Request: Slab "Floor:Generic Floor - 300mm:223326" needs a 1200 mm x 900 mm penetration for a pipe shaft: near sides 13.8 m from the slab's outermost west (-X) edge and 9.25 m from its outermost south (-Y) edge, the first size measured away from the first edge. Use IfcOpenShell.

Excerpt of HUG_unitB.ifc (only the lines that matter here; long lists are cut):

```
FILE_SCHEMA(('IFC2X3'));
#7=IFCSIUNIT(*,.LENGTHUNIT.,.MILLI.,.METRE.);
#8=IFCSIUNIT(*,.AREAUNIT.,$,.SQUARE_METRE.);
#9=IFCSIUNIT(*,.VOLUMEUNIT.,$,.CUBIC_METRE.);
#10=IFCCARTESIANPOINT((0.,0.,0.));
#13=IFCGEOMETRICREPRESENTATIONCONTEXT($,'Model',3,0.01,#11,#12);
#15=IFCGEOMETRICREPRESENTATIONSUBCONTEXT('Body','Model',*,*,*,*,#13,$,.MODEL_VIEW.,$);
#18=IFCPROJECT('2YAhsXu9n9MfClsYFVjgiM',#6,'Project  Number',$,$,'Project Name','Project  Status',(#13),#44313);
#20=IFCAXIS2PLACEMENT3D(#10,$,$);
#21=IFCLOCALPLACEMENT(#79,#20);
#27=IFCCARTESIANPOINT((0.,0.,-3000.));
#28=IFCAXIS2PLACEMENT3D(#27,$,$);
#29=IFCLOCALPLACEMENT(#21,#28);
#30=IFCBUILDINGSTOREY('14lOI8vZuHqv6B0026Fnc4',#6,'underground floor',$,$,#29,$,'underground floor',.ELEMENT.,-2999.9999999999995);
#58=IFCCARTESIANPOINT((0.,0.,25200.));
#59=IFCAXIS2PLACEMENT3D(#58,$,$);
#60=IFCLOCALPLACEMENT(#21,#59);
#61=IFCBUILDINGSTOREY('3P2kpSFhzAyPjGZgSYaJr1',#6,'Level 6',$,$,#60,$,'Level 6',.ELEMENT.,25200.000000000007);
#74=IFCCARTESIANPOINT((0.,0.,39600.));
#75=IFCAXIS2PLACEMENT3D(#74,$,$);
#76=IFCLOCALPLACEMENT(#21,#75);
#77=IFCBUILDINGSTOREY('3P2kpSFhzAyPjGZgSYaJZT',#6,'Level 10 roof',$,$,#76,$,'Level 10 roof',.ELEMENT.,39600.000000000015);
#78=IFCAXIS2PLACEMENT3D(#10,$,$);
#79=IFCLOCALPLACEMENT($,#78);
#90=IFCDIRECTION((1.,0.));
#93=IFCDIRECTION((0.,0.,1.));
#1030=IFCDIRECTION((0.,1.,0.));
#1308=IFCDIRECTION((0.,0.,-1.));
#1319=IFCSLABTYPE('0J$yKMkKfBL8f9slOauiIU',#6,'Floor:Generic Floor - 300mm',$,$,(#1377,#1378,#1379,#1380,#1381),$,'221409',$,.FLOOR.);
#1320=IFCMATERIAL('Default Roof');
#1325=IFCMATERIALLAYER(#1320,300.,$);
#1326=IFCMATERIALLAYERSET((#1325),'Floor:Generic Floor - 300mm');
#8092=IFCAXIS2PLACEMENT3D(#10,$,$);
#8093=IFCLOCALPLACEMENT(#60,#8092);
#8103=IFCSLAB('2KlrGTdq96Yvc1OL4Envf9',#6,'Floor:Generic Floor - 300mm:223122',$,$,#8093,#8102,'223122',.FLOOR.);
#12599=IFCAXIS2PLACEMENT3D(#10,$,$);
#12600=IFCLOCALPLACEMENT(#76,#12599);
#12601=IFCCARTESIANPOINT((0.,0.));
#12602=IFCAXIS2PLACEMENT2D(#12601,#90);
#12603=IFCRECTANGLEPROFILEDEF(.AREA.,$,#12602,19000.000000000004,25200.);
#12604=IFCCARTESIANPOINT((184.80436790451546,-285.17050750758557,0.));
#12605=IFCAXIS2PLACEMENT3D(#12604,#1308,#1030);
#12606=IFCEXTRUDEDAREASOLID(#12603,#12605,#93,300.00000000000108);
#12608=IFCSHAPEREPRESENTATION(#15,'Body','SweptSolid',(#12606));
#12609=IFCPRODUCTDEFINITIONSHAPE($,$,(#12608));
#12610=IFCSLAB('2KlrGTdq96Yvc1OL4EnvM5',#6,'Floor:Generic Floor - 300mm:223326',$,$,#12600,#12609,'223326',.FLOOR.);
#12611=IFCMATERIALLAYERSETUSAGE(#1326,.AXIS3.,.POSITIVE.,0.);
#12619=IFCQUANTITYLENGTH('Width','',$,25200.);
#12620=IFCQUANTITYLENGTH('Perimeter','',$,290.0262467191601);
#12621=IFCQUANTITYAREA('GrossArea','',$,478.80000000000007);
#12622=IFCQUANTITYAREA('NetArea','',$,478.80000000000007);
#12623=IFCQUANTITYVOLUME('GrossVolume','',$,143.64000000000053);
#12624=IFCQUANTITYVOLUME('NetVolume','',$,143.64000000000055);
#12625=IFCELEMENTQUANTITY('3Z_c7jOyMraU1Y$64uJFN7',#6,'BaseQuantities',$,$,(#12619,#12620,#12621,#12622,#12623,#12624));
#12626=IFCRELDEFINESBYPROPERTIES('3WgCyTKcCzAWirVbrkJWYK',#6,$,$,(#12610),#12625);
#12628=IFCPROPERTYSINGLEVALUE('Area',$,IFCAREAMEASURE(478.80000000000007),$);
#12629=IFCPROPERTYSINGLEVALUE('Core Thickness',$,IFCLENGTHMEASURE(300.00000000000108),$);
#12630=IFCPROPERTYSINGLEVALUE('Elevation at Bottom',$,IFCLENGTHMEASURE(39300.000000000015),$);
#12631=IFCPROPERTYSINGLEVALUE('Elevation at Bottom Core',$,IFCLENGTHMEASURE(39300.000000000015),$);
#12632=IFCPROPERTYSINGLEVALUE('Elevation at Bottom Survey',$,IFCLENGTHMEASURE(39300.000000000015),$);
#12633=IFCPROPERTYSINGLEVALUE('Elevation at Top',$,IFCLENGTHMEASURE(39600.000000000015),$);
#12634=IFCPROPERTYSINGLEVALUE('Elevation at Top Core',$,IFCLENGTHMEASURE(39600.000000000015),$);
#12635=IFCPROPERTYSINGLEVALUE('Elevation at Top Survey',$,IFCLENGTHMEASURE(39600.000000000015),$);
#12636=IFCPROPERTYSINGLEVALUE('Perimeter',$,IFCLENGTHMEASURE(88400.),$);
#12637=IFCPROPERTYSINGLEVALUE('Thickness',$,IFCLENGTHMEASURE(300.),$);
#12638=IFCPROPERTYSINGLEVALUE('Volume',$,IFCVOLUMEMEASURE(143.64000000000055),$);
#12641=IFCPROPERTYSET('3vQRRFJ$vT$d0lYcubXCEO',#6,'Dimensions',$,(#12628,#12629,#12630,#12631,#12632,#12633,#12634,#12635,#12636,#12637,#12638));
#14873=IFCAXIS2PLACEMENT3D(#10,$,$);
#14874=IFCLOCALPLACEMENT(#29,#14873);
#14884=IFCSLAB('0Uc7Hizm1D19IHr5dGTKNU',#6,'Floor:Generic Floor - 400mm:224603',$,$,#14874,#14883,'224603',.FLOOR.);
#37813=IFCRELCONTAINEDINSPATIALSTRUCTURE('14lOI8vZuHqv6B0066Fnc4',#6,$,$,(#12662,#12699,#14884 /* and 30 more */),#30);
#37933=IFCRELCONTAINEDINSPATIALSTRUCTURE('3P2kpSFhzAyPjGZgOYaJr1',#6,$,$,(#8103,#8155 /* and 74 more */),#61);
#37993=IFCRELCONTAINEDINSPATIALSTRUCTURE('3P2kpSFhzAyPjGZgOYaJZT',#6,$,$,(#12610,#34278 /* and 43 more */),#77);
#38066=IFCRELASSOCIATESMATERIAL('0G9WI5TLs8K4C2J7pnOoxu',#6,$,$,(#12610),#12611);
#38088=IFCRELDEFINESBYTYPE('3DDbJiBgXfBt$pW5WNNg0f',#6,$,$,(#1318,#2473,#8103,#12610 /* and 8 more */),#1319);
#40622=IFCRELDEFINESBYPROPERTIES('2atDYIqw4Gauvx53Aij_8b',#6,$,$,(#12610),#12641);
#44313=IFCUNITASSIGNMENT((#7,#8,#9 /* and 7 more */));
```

```python
import numpy as np
import ifcopenshell
import ifcopenshell.api.feature
import ifcopenshell.api.geometry
import ifcopenshell.api.pset
import ifcopenshell.api.root
import ifcopenshell.geom
import ifcopenshell.util.element
import ifcopenshell.util.placement
import ifcopenshell.util.representation
import ifcopenshell.util.shape
import ifcopenshell.util.unit

model = ifcopenshell.open("HUG_unitB.ifc")
unit_scale = ifcopenshell.util.unit.calculate_unit_scale(model)
area_scale = ifcopenshell.util.unit.calculate_unit_scale(model, "AREAUNIT")
volume_scale = ifcopenshell.util.unit.calculate_unit_scale(model, "VOLUMEUNIT")
settings = ifcopenshell.geom.settings()


def volume(element):
    """Net volume in cubic metres, openings subtracted."""
    shape = ifcopenshell.geom.create_shape(settings, element)
    return ifcopenshell.util.shape.get_volume(shape.geometry)


slab = model.by_guid("2KlrGTdq96Yvc1OL4EnvM5")
before = volume(slab)

# Extent in the slab's own axes, in metres. The edges named are its -X and -Y sides.
slab_shape = ifcopenshell.geom.create_shape(settings, slab)
vertices = ifcopenshell.util.shape.get_vertices(slab_shape.geometry)
x_min, y_min, bottom = vertices.min(axis=0)
top = vertices[:, 2].max()

opening = ifcopenshell.api.root.create_entity(model, ifc_class="IfcOpeningElement", name="Pipe shaft opening")
context = ifcopenshell.util.representation.get_context(model, "Model", "Body", "MODEL_VIEW")
width, depth = 1.2, 0.9
outline = [(0.0, 0.0), (width, 0.0), (width, depth), (0.0, depth), (0.0, 0.0)]
# Overshoot both faces by 50 mm so the cut is clean.
shape = ifcopenshell.api.geometry.add_slab_representation(
    model, context=context, depth=top - bottom + 0.1, polyline=outline
)
ifcopenshell.api.geometry.assign_representation(model, product=opening, representation=shape)

matrix = ifcopenshell.util.placement.get_local_placement(slab.ObjectPlacement)
matrix[:, 3] = matrix @ np.append(np.array([x_min + 13.8, y_min + 9.25, bottom - 0.05]) / unit_scale, 1.0)
ifcopenshell.api.geometry.edit_object_placement(model, product=opening, matrix=matrix, is_si=False)
ifcopenshell.api.feature.add_feature(model, feature=opening, element=slab)

after = volume(slab)

# Update the slab's stored quantities.
qto = model.by_id(ifcopenshell.util.element.get_pset(slab, "BaseQuantities", should_inherit=False)["id"])
ifcopenshell.api.pset.edit_qto(model, qto=qto, properties={
    "NetArea": after / (top - bottom) / area_scale,
    "NetVolume": after / volume_scale,
})
pset = model.by_id(ifcopenshell.util.element.get_pset(slab, "Dimensions", should_inherit=False)["id"])
ifcopenshell.api.pset.edit_pset(model, pset=pset, properties={
    "Area": model.create_entity("IfcAreaMeasure", after / (top - bottom) / area_scale),
    "Volume": model.create_entity("IfcVolumeMeasure", after / volume_scale),
})

print(f"slab volume {before:.3f} -> {after:.3f} m3")

model.write("HUG_unitB-out.ifc")
```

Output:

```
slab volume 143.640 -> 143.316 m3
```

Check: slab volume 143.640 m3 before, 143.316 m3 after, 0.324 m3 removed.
